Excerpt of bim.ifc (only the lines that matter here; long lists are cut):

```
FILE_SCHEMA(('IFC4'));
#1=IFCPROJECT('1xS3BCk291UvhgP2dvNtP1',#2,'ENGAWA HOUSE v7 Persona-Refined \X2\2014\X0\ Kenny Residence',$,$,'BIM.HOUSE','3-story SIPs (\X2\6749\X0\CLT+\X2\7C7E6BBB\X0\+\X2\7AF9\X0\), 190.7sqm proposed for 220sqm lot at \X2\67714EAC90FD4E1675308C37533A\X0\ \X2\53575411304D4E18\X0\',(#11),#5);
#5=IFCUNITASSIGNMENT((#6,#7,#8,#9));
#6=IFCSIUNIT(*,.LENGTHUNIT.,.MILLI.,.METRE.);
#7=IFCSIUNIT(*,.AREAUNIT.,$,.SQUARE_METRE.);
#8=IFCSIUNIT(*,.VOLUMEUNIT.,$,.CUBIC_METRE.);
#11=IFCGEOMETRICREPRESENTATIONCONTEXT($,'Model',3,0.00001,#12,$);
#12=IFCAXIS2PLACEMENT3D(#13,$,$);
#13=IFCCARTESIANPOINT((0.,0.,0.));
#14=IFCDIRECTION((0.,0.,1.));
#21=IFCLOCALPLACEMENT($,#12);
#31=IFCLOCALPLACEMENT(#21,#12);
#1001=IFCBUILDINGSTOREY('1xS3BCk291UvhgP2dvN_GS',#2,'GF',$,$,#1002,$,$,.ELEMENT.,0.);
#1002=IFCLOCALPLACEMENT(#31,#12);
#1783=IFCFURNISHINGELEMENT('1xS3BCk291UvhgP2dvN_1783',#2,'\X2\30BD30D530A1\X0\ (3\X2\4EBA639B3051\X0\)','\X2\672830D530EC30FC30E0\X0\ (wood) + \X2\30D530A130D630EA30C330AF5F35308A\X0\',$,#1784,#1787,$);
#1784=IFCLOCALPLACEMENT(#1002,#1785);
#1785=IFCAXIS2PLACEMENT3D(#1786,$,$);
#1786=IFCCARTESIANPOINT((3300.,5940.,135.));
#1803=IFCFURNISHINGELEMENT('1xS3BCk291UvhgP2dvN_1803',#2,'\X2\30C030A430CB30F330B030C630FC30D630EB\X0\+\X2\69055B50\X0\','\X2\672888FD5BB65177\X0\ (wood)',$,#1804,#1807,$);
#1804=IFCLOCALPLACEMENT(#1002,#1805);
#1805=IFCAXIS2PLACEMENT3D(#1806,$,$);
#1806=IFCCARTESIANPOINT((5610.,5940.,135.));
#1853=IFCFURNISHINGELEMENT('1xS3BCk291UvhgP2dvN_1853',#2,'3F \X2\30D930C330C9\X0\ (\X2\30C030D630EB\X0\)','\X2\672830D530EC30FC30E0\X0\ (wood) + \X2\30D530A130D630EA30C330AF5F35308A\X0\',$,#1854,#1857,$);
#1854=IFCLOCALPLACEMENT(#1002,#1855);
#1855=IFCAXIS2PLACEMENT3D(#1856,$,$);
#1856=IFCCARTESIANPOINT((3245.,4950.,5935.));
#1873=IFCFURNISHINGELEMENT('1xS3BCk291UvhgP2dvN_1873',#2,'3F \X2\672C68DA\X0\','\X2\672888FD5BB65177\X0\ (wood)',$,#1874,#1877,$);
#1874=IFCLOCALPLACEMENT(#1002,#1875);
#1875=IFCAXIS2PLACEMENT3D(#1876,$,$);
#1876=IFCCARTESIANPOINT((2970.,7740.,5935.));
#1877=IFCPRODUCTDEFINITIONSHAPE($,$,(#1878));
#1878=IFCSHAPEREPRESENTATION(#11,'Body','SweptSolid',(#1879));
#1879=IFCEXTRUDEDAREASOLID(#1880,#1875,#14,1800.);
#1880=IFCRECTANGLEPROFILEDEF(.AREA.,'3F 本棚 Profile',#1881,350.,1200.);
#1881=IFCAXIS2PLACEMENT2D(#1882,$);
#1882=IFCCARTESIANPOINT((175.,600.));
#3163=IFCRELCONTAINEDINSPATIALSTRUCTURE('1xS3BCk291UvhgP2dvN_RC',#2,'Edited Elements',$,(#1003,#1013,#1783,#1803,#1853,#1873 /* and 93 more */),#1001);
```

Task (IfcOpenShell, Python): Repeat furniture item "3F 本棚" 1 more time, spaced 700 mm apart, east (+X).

```python
import numpy as np
import ifcopenshell
import ifcopenshell.api.geometry
import ifcopenshell.api.root
import ifcopenshell.util.element
import ifcopenshell.util.placement
import ifcopenshell.util.unit

model = ifcopenshell.open("bim.ifc")
unit_scale = ifcopenshell.util.unit.calculate_unit_scale(model)


def reuse_history(source, copy):
    """copy_class also copies each property set's owner history, people and application; keep the originals."""
    for rel in copy.IsDefinedBy:
        if rel.is_a("IfcRelDefinesByProperties") and (history := rel.RelatingPropertyDefinition.OwnerHistory):
            rel.RelatingPropertyDefinition.OwnerHistory = source.OwnerHistory
            ifcopenshell.util.element.remove_deep2(model, history)


source = model.by_guid("1xS3BCk291UvhgP2dvN_1873")
base = ifcopenshell.util.placement.get_local_placement(source.ObjectPlacement)
step = np.array([1.0, 0.0, 0.0]) * 0.7 / unit_scale

for i in range(1, 2):
    copy = ifcopenshell.api.root.copy_class(model, product=source)
    copy.Representation = ifcopenshell.util.element.copy_deep(
        model, source.Representation, exclude=["IfcGeometricRepresentationContext", "IfcRepresentationMap"]
    )
    reuse_history(source, copy)
    matrix = base.copy()
    matrix[:3, 3] += i * step
    print("added at", matrix[:3, 3].round(3) + 0.0)
    ifcopenshell.api.geometry.edit_object_placement(model, product=copy, matrix=matrix, is_si=False)

model.write("bim_v2.ifc")
```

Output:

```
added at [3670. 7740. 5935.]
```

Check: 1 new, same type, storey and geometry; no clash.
